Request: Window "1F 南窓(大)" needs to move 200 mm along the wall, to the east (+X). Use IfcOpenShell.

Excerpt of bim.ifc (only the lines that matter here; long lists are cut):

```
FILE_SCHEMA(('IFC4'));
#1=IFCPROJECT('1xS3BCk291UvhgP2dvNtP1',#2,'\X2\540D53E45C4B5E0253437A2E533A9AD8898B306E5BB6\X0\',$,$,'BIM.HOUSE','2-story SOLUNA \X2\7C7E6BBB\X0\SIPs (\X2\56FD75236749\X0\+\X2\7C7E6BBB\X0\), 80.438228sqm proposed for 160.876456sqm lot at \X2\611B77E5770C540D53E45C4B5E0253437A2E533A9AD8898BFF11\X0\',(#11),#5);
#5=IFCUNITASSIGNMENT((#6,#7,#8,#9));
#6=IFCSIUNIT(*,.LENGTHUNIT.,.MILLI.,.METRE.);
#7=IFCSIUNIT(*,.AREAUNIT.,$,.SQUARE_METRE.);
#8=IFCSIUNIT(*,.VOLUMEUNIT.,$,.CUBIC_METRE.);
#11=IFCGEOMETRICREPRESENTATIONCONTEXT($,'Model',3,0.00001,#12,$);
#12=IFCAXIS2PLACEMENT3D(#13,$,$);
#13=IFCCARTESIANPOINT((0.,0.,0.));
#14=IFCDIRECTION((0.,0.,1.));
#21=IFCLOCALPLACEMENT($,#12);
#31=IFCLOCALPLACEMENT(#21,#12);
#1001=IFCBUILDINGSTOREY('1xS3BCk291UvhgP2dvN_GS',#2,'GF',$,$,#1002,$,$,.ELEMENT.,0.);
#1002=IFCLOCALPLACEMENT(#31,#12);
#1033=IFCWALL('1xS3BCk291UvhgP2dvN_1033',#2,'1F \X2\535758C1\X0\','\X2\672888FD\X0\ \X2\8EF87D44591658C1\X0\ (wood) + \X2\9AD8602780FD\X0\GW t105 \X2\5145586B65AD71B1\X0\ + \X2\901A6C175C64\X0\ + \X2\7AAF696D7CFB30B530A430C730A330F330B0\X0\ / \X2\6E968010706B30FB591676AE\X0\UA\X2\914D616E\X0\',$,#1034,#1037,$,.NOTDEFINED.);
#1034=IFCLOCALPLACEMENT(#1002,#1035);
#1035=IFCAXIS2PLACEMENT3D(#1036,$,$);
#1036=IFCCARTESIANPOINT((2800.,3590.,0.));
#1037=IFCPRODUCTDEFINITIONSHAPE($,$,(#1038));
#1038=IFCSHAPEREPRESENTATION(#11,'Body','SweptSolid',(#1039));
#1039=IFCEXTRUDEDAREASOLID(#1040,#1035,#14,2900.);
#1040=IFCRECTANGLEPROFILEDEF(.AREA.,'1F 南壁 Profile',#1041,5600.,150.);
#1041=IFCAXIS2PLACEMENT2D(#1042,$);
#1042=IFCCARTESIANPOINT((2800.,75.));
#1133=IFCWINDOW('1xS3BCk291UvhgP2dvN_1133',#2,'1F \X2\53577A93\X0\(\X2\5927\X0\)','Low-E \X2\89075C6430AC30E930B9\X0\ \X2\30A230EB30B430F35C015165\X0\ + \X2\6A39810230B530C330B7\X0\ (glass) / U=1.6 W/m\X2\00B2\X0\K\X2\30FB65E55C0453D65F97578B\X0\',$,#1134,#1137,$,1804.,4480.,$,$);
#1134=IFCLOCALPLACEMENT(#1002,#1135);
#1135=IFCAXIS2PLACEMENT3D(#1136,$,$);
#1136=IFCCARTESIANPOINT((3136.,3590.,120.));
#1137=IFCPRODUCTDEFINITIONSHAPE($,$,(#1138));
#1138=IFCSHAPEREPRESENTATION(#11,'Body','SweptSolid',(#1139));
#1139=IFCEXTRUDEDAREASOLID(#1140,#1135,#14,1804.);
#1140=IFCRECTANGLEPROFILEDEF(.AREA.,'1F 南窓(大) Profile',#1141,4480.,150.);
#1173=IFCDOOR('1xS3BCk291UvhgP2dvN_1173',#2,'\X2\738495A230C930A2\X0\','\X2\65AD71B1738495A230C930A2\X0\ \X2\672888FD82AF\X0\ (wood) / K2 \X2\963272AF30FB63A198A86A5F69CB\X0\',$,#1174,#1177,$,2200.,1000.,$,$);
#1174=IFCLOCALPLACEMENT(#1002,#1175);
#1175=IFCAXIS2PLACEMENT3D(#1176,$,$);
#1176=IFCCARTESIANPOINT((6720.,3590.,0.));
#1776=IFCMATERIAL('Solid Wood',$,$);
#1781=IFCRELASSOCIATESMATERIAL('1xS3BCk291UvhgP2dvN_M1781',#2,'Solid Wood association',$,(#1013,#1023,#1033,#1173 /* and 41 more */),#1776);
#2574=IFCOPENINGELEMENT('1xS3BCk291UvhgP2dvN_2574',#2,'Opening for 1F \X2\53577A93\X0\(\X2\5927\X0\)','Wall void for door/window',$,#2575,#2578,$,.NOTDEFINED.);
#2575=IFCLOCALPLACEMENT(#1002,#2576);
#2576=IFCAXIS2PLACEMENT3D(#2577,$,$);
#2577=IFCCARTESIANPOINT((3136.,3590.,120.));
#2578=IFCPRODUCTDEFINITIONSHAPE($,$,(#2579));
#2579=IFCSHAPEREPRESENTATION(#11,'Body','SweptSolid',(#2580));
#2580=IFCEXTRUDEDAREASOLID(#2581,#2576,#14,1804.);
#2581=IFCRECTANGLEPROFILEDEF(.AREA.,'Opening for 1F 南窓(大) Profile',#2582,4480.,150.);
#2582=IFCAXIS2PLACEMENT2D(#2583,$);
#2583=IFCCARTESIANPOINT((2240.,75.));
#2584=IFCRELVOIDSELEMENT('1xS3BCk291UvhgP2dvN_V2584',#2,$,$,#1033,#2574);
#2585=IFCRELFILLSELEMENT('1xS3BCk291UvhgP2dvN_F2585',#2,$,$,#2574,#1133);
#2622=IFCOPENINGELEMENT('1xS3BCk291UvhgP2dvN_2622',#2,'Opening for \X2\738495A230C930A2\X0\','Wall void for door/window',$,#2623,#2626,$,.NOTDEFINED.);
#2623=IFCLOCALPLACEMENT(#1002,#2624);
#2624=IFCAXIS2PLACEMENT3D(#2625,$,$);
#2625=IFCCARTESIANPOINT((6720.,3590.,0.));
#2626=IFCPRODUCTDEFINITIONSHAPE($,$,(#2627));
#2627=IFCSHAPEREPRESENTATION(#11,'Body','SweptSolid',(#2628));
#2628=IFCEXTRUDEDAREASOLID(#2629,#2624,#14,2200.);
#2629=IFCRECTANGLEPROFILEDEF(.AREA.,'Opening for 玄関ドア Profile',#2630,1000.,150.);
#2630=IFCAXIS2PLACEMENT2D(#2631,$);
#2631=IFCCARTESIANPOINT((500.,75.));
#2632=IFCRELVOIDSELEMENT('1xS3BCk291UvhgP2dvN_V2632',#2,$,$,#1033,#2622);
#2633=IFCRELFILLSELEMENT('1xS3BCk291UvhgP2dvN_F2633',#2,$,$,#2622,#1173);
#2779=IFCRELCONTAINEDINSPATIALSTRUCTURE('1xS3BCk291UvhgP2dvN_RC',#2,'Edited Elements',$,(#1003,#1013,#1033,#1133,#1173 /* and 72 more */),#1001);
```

```python
import ifcopenshell
import ifcopenshell.api.geometry
import ifcopenshell.util.placement
import ifcopenshell.util.unit

model = ifcopenshell.open("bim.ifc")
unit_scale = ifcopenshell.util.unit.calculate_unit_scale(model)

window = model.by_guid("1xS3BCk291UvhgP2dvN_1133")
opening = window.FillsVoids[0].RelatingOpeningElement
wall = opening.VoidsElements[0].RelatingBuildingElement

wall_matrix = ifcopenshell.util.placement.get_local_placement(wall.ObjectPlacement)
shift = wall_matrix[:3, 0] * 0.2 / unit_scale
before = ifcopenshell.util.placement.get_local_placement(window.ObjectPlacement)[:3, 3].copy()

# The window is not placed relative to its opening, so move both.
for product in (opening, window):
    matrix = ifcopenshell.util.placement.get_local_placement(product.ObjectPlacement)
    matrix[:3, 3] += shift
    ifcopenshell.api.geometry.edit_object_placement(model, product=product, matrix=matrix, is_si=False)

after = ifcopenshell.util.placement.get_local_placement(window.ObjectPlacement)[:3, 3]
print("window moved by", (after - before).round(3) + 0.0)

model.write("bim_updated.ifc")
```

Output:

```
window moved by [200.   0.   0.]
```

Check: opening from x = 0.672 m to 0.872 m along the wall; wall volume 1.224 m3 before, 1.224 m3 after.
